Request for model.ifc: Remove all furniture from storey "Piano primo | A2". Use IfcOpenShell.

First a look at what the model holds.

```python
import ifcopenshell
import ifcopenshell.util.element

model = ifcopenshell.open("model.ifc")
print(model.schema)
storey = next(s for s in model.by_type("IfcBuildingStorey") if s.Name == "Piano primo | A2")
furniture = [e for e in ifcopenshell.util.element.get_decomposition(storey) if e.is_a("IfcFurnishingElement")]
seen = {}
for e in furniture:
    element_type = ifcopenshell.util.element.get_type(e)
    name = element_type.Name if element_type not in (None, e) else None
    seen[name] = seen.get(name, 0) + 1
for name, count in sorted(seen.items(), key=str):
    print(count, "x", name)
```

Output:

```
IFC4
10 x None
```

```python
import ifcopenshell
import ifcopenshell.api.root
import ifcopenshell.util.element

model = ifcopenshell.open("model.ifc")

storey = next(s for s in model.by_type("IfcBuildingStorey") if s.Name == "Piano primo | A2")
furniture = [e for e in ifcopenshell.util.element.get_decomposition(storey) if e.is_a("IfcFurnishingElement")]

for e in furniture:
    ifcopenshell.api.root.remove_product(model, product=e)
print(len(furniture), "removed")

model.write("model-out.ifc")
```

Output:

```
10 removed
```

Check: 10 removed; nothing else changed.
